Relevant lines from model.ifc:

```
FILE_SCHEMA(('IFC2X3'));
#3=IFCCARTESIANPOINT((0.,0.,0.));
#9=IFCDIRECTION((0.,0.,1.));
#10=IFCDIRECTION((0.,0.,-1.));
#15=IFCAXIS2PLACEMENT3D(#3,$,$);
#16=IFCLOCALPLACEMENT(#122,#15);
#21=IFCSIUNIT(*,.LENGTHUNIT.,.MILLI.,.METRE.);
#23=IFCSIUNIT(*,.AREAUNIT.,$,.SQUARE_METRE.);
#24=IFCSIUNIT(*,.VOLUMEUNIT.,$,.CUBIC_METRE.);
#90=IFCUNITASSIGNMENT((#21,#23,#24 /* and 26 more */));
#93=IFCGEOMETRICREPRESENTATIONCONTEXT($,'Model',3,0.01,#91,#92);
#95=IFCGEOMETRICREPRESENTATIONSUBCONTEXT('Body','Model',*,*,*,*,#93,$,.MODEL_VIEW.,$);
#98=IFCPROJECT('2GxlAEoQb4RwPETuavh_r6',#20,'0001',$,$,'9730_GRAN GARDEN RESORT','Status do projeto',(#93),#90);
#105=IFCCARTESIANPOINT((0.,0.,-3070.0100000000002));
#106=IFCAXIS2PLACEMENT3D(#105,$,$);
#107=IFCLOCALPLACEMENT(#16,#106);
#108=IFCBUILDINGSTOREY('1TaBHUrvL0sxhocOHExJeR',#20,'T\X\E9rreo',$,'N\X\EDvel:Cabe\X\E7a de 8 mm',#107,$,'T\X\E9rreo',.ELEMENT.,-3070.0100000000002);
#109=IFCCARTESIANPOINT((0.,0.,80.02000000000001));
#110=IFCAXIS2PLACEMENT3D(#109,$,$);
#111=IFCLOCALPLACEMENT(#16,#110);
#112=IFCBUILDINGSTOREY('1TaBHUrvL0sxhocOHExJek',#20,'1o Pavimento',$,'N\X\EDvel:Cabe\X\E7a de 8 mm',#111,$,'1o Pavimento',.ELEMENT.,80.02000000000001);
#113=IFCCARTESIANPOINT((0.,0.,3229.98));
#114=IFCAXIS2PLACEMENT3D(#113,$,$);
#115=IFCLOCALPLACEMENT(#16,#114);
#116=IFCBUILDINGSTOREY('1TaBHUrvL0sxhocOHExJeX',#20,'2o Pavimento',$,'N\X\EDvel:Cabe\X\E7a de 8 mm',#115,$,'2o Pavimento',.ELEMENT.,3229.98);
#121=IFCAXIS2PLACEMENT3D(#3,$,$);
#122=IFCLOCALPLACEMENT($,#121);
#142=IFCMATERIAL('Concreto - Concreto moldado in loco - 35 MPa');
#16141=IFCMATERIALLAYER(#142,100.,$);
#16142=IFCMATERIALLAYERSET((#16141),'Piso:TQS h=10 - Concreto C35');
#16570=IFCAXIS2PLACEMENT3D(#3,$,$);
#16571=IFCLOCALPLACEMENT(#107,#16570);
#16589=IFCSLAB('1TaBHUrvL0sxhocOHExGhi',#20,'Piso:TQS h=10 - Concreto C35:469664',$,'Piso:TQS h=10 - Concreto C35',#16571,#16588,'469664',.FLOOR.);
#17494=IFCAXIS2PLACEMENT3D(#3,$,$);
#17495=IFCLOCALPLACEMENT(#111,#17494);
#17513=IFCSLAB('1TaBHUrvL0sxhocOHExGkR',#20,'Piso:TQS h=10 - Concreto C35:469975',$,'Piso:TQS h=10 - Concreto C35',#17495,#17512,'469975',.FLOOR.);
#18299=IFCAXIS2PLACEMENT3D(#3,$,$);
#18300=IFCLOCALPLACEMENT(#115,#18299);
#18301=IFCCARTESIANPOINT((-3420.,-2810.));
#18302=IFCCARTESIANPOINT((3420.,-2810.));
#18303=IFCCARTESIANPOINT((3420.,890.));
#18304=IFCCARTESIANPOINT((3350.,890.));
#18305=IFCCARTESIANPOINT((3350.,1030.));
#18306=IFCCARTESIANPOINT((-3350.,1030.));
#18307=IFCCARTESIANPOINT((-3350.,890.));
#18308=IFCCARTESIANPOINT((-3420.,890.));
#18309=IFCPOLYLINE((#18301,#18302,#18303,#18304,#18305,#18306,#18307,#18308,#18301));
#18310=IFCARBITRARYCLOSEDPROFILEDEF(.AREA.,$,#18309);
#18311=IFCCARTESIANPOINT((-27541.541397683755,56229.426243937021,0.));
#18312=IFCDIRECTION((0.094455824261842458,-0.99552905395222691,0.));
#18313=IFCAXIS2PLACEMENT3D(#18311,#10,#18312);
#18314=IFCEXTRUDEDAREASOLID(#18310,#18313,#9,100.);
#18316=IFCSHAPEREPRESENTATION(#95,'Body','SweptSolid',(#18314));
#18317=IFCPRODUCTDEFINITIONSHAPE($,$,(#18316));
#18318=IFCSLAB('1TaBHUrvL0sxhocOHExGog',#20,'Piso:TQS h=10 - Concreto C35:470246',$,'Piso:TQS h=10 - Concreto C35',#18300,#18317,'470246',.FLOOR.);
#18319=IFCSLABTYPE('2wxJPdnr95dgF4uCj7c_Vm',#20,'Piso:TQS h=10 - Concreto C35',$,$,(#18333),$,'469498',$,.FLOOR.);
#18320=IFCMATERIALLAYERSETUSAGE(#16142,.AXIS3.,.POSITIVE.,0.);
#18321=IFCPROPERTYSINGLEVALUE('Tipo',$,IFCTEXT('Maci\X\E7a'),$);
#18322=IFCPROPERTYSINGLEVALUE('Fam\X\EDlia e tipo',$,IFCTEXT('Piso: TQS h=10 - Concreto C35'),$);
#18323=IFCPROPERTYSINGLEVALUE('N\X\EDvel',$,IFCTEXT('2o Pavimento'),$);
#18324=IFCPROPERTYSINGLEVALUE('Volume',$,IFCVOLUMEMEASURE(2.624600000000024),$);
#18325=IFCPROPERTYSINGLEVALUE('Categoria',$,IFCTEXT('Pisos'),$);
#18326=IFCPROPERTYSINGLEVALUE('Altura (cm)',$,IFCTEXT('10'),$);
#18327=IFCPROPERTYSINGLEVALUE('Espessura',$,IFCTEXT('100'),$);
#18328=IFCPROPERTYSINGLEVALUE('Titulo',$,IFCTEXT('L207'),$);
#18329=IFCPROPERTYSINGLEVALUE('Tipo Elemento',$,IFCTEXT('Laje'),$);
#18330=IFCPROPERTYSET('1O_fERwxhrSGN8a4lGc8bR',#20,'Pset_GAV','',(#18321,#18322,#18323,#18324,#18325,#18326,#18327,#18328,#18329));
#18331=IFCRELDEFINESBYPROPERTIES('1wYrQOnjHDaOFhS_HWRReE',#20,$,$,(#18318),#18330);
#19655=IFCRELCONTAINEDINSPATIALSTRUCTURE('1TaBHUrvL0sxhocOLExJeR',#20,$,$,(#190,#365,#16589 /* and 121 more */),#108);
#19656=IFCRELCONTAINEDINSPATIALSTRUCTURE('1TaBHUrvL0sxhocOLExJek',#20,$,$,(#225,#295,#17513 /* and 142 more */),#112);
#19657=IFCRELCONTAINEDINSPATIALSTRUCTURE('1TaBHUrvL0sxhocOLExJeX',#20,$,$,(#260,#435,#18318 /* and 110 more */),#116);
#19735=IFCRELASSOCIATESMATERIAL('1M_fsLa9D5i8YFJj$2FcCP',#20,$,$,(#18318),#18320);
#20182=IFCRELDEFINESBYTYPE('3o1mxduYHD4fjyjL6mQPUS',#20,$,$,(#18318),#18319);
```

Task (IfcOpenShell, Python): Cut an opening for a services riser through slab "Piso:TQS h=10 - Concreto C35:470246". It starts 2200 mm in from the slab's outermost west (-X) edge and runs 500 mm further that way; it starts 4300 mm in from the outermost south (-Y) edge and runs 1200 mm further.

```python
import numpy as np
import ifcopenshell
import ifcopenshell.api.feature
import ifcopenshell.api.geometry
import ifcopenshell.api.pset
import ifcopenshell.api.root
import ifcopenshell.geom
import ifcopenshell.util.element
import ifcopenshell.util.placement
import ifcopenshell.util.representation
import ifcopenshell.util.shape
import ifcopenshell.util.unit

model = ifcopenshell.open("model.ifc")
unit_scale = ifcopenshell.util.unit.calculate_unit_scale(model)
volume_scale = ifcopenshell.util.unit.calculate_unit_scale(model, "VOLUMEUNIT")
settings = ifcopenshell.geom.settings()


def volume(element):
    """Net volume in cubic metres, openings subtracted."""
    shape = ifcopenshell.geom.create_shape(settings, element)
    return ifcopenshell.util.shape.get_volume(shape.geometry)


slab = model.by_guid("1TaBHUrvL0sxhocOHExGog")
before = volume(slab)

# Extent in the slab's own axes, in metres. The edges named are its -X and -Y sides.
slab_shape = ifcopenshell.geom.create_shape(settings, slab)
vertices = ifcopenshell.util.shape.get_vertices(slab_shape.geometry)
x_min, y_min, bottom = vertices.min(axis=0)
top = vertices[:, 2].max()

opening = ifcopenshell.api.root.create_entity(model, ifc_class="IfcOpeningElement", name="Services riser opening")
context = ifcopenshell.util.representation.get_context(model, "Model", "Body", "MODEL_VIEW")
width, depth = 0.5, 1.2
outline = [(0.0, 0.0), (width, 0.0), (width, depth), (0.0, depth), (0.0, 0.0)]
# Overshoot both faces by 50 mm so the cut is clean.
shape = ifcopenshell.api.geometry.add_slab_representation(
    model, context=context, depth=top - bottom + 0.1, polyline=outline
)
ifcopenshell.api.geometry.assign_representation(model, product=opening, representation=shape)

matrix = ifcopenshell.util.placement.get_local_placement(slab.ObjectPlacement)
matrix[:, 3] = matrix @ np.append(np.array([x_min + 2.2, y_min + 4.3, bottom - 0.05]) / unit_scale, 1.0)
ifcopenshell.api.geometry.edit_object_placement(model, product=opening, matrix=matrix, is_si=False)
ifcopenshell.api.feature.add_feature(model, feature=opening, element=slab)

after = volume(slab)

# Update the slab's stored quantities.
pset = model.by_id(ifcopenshell.util.element.get_pset(slab, "Pset_GAV", should_inherit=False)["id"])
ifcopenshell.api.pset.edit_pset(model, pset=pset, properties={
    "Volume": model.create_entity("IfcVolumeMeasure", after / volume_scale),
})

print(f"slab volume {before:.3f} -> {after:.3f} m3")

model.write("model_edited.ifc")
```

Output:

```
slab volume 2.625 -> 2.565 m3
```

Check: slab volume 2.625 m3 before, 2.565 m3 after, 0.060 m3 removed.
